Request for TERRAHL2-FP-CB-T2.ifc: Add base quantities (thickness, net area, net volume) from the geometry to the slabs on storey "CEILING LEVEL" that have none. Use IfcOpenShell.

First a look at what the model holds.

```python
import ifcopenshell
import ifcopenshell.util.element
import ifcopenshell.util.unit

model = ifcopenshell.open("TERRAHL2-FP-CB-T2.ifc")
print(model.schema)
for unit_type in ("LENGTHUNIT", "AREAUNIT", "VOLUMEUNIT"):
    print(unit_type, ifcopenshell.util.unit.calculate_unit_scale(model, unit_type))
storey = next(s for s in model.by_type("IfcBuildingStorey") if s.Name == "CEILING LEVEL")
slabs = [e for e in ifcopenshell.util.element.get_decomposition(storey) if e.is_a("IfcSlab")]
for e in sorted(slabs, key=lambda e: e.id()):
    print(e.id(), e.is_a(), e.Name, list(ifcopenshell.util.element.get_psets(e, qtos_only=True)), sep=" | ")
```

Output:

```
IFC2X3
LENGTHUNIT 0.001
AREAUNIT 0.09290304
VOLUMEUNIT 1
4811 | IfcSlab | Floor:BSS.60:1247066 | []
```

```python
import ifcopenshell
import ifcopenshell.api.pset
import ifcopenshell.geom
import ifcopenshell.util.element
import ifcopenshell.util.shape
import ifcopenshell.util.unit

model = ifcopenshell.open("TERRAHL2-FP-CB-T2.ifc")
unit_scale = ifcopenshell.util.unit.calculate_unit_scale(model)
area_scale = ifcopenshell.util.unit.calculate_unit_scale(model, "AREAUNIT")
volume_scale = ifcopenshell.util.unit.calculate_unit_scale(model, "VOLUMEUNIT")
settings = ifcopenshell.geom.settings()

storey = next(s for s in model.by_type("IfcBuildingStorey") if s.Name == "CEILING LEVEL")
slabs = [e for e in ifcopenshell.util.element.get_decomposition(storey) if e.is_a("IfcSlab")]

for e in sorted(slabs, key=lambda e: e.id()):
    if ifcopenshell.util.element.get_psets(e, qtos_only=True, should_inherit=False):
        continue
    # Geometry comes back in metres, in the element's own axes.
    shape = ifcopenshell.geom.create_shape(settings, e)
    values = {
        "Width": ifcopenshell.util.shape.get_z(shape.geometry) / unit_scale,
        "NetArea": ifcopenshell.util.shape.get_footprint_area(shape.geometry) / area_scale,
        "NetVolume": ifcopenshell.util.shape.get_volume(shape.geometry) / volume_scale,
    }
    qto = ifcopenshell.api.pset.add_qto(model, product=e, name="BaseQuantities")
    ifcopenshell.api.pset.edit_qto(model, qto=qto, properties=values)
    print(e.id(), {k: round(v, 3) for k, v in values.items()})

model.write("TERRAHL2-FP-CB-T2-out.ifc")
```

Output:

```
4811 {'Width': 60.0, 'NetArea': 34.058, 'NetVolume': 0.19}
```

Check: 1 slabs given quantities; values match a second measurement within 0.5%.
